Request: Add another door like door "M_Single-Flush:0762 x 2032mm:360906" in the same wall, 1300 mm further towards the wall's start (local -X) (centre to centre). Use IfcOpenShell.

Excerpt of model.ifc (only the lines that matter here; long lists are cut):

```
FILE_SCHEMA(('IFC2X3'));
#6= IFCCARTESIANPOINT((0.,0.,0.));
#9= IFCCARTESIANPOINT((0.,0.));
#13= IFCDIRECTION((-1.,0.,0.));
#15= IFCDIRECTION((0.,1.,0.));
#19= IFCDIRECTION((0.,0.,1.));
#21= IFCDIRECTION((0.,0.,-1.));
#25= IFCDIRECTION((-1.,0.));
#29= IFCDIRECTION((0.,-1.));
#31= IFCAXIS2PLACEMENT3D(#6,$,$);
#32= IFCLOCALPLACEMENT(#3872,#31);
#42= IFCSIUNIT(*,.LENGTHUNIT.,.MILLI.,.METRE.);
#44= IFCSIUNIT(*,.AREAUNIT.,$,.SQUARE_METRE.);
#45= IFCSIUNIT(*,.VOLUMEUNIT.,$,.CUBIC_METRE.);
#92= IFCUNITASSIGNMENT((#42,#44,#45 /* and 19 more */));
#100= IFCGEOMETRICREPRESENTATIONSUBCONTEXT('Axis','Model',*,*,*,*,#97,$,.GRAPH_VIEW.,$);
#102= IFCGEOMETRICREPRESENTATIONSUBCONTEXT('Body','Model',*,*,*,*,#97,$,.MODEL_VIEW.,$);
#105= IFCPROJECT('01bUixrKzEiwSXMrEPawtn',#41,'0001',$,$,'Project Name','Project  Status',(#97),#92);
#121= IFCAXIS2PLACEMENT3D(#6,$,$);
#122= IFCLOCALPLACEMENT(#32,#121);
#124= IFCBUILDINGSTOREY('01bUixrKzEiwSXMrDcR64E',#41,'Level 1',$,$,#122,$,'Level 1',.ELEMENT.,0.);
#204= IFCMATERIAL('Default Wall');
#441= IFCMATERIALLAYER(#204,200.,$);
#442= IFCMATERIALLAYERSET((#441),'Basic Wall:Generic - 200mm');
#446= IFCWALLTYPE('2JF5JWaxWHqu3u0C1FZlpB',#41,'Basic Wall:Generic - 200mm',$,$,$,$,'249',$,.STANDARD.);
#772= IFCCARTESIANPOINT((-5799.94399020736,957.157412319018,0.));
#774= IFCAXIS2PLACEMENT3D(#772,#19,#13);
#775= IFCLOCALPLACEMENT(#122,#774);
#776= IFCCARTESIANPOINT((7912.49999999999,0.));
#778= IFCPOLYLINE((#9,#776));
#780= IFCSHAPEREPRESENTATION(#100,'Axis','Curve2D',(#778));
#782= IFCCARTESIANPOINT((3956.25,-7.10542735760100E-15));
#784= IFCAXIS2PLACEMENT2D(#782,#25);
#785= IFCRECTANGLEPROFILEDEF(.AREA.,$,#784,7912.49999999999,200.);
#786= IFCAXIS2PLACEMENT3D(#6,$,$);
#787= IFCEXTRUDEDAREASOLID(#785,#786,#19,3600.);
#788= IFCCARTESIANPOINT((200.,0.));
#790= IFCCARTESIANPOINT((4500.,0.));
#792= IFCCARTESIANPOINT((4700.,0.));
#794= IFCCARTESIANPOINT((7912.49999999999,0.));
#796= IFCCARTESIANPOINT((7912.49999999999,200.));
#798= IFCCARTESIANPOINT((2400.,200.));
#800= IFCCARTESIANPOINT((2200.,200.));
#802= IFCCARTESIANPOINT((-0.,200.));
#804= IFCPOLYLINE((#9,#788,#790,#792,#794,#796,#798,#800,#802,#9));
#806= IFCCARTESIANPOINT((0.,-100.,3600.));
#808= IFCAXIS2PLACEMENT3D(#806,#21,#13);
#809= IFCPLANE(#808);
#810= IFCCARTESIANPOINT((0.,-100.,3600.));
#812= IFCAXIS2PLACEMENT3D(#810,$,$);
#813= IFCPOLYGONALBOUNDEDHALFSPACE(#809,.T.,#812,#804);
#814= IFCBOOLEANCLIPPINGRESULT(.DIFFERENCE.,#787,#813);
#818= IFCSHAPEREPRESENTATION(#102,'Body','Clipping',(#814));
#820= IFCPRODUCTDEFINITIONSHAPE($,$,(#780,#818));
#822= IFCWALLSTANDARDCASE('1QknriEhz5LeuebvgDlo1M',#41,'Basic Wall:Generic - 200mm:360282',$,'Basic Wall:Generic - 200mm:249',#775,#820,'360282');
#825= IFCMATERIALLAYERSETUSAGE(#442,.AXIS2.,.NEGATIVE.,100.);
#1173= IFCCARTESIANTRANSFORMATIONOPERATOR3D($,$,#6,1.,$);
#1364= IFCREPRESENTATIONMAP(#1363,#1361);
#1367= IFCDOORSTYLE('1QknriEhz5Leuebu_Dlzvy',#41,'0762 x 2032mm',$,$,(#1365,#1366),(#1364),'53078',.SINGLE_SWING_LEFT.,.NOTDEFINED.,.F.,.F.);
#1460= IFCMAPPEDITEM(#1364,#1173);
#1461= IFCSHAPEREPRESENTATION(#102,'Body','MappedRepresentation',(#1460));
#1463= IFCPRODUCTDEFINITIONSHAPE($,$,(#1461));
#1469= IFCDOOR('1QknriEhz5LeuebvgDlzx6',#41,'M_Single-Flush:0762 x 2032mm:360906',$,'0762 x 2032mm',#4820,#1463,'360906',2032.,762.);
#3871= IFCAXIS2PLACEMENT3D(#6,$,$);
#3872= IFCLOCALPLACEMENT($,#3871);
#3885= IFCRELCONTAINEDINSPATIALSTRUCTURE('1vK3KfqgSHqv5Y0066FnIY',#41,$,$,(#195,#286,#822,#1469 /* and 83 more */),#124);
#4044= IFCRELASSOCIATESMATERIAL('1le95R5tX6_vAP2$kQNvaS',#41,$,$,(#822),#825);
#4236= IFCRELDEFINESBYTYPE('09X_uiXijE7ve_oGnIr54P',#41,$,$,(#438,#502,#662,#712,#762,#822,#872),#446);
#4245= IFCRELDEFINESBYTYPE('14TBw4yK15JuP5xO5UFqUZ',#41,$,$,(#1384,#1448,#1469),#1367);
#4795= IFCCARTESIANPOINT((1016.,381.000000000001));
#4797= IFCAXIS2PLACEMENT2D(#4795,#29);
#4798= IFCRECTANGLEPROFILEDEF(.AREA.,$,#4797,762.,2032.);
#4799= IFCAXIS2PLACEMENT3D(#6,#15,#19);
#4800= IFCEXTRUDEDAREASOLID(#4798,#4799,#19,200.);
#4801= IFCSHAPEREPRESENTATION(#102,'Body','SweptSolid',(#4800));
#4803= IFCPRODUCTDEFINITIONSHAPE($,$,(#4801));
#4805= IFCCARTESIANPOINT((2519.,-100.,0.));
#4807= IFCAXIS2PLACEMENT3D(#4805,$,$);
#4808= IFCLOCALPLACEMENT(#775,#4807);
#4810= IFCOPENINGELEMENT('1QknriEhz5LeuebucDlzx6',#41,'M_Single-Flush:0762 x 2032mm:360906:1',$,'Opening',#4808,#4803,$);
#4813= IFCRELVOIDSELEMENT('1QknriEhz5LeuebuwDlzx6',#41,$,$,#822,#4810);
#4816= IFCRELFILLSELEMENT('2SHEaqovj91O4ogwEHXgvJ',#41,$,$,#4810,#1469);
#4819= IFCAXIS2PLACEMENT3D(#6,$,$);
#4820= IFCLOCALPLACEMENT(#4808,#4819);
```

```python
import ifcopenshell
import ifcopenshell.api.feature
import ifcopenshell.api.geometry
import ifcopenshell.api.root
import ifcopenshell.geom
import ifcopenshell.util.element
import ifcopenshell.util.placement
import ifcopenshell.util.shape
import ifcopenshell.util.unit

model = ifcopenshell.open("model.ifc")
unit_scale = ifcopenshell.util.unit.calculate_unit_scale(model)
settings = ifcopenshell.geom.settings()


def volume(element):
    """Net volume in cubic metres, openings subtracted."""
    shape = ifcopenshell.geom.create_shape(settings, element)
    return ifcopenshell.util.shape.get_volume(shape.geometry)


def reuse_history(source, copy):
    """copy_class also copies each property set's owner history, people and application; keep the originals."""
    for rel in copy.IsDefinedBy:
        if rel.is_a("IfcRelDefinesByProperties") and (history := rel.RelatingPropertyDefinition.OwnerHistory):
            rel.RelatingPropertyDefinition.OwnerHistory = source.OwnerHistory
            ifcopenshell.util.element.remove_deep2(model, history)


door = model.by_guid("1QknriEhz5LeuebvgDlzx6")
opening = door.FillsVoids[0].RelatingOpeningElement
wall = opening.VoidsElements[0].RelatingBuildingElement
before = volume(wall)
shift = ifcopenshell.util.placement.get_local_placement(wall.ObjectPlacement)[:3, 0] * -1.3 / unit_scale

# copy_class copies the void relationship, type, container and properties, but no geometry.
new_opening = ifcopenshell.api.root.copy_class(model, product=opening)
new_opening.Representation = ifcopenshell.util.element.copy_deep(
    model, opening.Representation, exclude=["IfcGeometricRepresentationContext", "IfcRepresentationMap"]
)
new_opening.Name = "M_Single-Flush:0762 x 2032mm"
new_door = ifcopenshell.api.root.copy_class(model, product=door)
new_door.Representation = ifcopenshell.util.element.copy_deep(
    model, door.Representation, exclude=["IfcGeometricRepresentationContext", "IfcRepresentationMap"]
)
new_door.Name = "M_Single-Flush:0762 x 2032mm"
new_door.Tag = None
reuse_history(door, new_door)
fills = ifcopenshell.api.feature.add_filling(model, opening=new_opening, element=new_door)
fills.OwnerHistory = new_door.OwnerHistory  # required in IFC2X3

for old, new in ((opening, new_opening), (door, new_door)):
    matrix = ifcopenshell.util.placement.get_local_placement(old.ObjectPlacement)
    matrix[:3, 3] += shift
    ifcopenshell.api.geometry.edit_object_placement(model, product=new, matrix=matrix, is_si=False)

after = volume(wall)

print(f"wall volume {before:.3f} -> {after:.3f} m3")

model.write("model_v2.ifc")
```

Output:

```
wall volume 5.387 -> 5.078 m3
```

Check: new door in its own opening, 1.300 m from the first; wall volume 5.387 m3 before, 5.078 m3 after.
